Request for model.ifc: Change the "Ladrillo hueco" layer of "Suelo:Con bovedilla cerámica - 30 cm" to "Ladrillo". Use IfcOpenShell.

First a look at what the model holds.

```python
import ifcopenshell
import ifcopenshell.util.element

model = ifcopenshell.open("model.ifc")
print(model.schema)
for layer_set in model.by_type("IfcMaterialLayerSet"):
    if layer_set.LayerSetName == "Suelo:Con bovedilla cerámica - 30 cm":
        for layer in layer_set.MaterialLayers:
            print(layer.id(), layer.Material and layer.Material.Name, layer.LayerThickness, sep=" | ")
        print(len(ifcopenshell.util.element.get_elements_by_material(model, layer_set)), "elements and types use it")
print(sorted(m.Name for m in model.by_type("IfcMaterial") if m.Name)[:60])
```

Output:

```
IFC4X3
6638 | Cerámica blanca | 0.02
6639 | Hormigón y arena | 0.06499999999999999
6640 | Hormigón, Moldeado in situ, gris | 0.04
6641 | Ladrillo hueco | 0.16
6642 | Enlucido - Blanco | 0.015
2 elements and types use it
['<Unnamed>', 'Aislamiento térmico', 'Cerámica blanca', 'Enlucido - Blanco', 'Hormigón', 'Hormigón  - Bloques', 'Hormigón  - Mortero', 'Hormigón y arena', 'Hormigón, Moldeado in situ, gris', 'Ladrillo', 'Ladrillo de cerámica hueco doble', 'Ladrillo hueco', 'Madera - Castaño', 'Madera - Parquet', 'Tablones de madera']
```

```python
import ifcopenshell
import ifcopenshell.api.material

model = ifcopenshell.open("model.ifc")

layer_set = next(s for s in model.by_type("IfcMaterialLayerSet") if s.LayerSetName == "Suelo:Con bovedilla cerámica - 30 cm")
layer = next(l for l in layer_set.MaterialLayers if l.Material and l.Material.Name == "Ladrillo hueco")
material = next(m for m in model.by_type("IfcMaterial") if m.Name == "Ladrillo")

# Point this one layer at the other material; renaming the old one would change it everywhere.
ifcopenshell.api.material.edit_layer(model, layer=layer, attributes={"Name": material.Name}, material=material)

print([l.Material.Name if l.Material else None for l in layer_set.MaterialLayers])

model.write("model_rev.ifc")
```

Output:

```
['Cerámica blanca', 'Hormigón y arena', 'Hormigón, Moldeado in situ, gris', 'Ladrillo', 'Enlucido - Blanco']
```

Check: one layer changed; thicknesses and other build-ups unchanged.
